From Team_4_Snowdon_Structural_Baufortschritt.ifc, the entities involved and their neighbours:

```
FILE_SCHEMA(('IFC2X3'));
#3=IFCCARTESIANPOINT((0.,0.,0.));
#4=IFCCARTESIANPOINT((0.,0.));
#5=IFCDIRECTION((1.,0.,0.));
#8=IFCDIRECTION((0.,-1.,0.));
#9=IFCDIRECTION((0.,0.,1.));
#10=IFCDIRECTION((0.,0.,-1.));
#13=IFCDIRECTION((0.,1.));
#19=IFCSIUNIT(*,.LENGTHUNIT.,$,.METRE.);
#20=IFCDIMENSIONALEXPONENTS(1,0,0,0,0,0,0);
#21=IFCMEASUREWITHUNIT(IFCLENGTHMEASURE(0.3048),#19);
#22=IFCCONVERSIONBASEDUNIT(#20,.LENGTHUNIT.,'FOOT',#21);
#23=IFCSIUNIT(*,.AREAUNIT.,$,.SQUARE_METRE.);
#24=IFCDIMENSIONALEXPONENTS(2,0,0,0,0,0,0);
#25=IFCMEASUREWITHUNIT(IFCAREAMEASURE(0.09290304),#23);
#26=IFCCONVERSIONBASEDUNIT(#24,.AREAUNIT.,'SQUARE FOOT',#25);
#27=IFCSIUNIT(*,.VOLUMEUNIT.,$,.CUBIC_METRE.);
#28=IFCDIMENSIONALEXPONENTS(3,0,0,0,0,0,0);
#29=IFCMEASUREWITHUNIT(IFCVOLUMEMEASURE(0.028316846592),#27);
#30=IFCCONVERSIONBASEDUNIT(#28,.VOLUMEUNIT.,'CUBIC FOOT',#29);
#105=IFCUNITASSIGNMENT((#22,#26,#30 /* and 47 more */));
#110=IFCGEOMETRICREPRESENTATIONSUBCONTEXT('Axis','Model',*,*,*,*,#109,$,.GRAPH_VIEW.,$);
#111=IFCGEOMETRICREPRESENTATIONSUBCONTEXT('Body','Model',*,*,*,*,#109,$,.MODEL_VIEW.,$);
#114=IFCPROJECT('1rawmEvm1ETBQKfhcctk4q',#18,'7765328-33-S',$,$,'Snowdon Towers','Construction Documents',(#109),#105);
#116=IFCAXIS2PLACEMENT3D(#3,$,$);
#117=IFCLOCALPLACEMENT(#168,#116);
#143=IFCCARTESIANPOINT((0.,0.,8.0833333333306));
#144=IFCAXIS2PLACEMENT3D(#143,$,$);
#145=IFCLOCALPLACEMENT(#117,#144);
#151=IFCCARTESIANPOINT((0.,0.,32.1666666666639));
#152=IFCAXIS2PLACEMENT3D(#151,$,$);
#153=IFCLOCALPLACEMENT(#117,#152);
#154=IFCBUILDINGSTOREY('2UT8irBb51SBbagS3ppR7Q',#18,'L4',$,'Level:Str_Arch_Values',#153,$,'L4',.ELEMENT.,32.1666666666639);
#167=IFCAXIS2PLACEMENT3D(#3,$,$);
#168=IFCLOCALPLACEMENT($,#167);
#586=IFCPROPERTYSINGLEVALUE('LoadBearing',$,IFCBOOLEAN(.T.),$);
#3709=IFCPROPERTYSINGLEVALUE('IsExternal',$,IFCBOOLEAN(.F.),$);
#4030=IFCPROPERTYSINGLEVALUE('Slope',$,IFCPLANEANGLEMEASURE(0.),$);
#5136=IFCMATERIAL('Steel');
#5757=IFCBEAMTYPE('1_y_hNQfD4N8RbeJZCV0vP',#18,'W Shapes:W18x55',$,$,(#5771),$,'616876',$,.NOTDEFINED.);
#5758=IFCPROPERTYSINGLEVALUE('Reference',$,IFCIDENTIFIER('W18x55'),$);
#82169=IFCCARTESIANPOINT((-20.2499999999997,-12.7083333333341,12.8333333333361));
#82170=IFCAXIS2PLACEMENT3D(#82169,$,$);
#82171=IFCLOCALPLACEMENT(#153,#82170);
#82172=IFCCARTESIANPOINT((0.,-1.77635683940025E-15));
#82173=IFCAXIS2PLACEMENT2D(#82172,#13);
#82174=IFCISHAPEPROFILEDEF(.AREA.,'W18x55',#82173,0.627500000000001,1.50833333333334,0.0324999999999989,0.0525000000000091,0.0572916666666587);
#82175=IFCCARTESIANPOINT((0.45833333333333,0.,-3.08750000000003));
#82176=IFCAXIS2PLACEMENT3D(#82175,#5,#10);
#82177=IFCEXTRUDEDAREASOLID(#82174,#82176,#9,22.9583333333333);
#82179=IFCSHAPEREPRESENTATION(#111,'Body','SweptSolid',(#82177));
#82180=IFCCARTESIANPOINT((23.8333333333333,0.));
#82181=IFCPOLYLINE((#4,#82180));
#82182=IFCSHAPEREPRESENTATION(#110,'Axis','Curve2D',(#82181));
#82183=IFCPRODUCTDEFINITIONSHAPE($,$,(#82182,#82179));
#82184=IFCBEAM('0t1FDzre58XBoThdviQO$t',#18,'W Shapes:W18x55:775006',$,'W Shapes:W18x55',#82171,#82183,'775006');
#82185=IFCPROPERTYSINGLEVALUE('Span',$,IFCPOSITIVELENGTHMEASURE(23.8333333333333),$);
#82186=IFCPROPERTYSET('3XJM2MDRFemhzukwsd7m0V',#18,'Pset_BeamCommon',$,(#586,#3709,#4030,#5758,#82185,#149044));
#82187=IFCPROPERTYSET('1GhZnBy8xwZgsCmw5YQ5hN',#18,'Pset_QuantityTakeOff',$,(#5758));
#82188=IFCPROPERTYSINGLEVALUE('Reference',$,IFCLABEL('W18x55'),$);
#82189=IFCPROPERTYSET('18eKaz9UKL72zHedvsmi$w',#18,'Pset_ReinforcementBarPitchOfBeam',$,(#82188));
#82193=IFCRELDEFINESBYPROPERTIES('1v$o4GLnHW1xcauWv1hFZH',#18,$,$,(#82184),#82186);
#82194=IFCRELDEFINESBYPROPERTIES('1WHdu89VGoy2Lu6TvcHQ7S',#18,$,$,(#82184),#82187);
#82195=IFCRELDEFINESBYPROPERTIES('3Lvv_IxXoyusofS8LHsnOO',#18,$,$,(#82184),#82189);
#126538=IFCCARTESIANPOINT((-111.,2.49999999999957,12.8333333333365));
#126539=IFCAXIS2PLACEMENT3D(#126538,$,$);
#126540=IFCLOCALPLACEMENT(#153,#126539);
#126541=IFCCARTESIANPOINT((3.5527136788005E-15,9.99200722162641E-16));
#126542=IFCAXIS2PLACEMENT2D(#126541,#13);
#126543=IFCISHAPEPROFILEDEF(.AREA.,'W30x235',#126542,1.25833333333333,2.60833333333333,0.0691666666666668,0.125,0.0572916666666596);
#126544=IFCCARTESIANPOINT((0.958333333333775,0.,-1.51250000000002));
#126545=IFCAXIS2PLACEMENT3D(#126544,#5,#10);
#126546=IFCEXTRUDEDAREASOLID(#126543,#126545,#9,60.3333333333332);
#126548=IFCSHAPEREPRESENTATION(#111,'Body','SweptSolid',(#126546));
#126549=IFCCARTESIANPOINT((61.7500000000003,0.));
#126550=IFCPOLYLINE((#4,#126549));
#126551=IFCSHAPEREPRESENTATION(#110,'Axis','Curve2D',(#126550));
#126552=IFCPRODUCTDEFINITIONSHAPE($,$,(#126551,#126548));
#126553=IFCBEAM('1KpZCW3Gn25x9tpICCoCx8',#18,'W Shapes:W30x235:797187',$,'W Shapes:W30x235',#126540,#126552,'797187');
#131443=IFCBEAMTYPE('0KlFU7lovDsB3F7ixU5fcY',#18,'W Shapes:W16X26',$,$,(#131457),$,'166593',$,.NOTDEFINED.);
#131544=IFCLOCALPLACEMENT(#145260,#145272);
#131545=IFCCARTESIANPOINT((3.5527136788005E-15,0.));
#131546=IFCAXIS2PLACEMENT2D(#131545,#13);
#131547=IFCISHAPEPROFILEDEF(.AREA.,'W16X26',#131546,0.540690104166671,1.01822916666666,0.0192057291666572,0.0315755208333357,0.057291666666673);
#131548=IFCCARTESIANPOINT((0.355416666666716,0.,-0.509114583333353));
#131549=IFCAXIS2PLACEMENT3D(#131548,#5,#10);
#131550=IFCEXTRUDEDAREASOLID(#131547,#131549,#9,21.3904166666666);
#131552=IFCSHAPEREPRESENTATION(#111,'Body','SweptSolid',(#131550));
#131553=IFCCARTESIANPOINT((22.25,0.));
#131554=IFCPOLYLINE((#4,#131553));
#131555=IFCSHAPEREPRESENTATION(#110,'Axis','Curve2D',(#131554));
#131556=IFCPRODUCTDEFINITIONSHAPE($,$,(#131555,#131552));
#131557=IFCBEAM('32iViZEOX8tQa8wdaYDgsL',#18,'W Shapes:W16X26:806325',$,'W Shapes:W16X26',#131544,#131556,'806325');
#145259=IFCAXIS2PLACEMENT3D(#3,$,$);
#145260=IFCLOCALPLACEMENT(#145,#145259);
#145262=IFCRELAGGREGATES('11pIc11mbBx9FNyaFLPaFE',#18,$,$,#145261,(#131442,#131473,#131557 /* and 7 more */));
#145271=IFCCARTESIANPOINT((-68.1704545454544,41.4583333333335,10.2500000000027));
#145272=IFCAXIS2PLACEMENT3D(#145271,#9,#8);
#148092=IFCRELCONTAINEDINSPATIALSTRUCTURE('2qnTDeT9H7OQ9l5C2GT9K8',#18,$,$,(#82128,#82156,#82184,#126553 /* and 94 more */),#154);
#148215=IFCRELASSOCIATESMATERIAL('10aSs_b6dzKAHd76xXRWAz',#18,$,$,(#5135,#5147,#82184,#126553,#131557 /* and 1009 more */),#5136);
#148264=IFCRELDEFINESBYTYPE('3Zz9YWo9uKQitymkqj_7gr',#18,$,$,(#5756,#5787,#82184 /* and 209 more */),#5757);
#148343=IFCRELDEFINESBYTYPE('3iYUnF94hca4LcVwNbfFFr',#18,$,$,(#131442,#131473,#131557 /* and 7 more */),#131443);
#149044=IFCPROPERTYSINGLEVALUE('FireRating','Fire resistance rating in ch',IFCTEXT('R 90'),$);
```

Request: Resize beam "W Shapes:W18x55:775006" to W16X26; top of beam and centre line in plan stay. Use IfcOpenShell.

```python
import ifcopenshell
import ifcopenshell.api.pset
import ifcopenshell.api.type
import ifcopenshell.util.element
import ifcopenshell.util.representation

model = ifcopenshell.open("Team_4_Snowdon_Structural_Baufortschritt.ifc")

member = model.by_guid("0t1FDzre58XBoThdviQO$t")
source = next(p for p in model.by_type("IfcIShapeProfileDef") if p.ProfileName == "W16X26")

body = ifcopenshell.util.representation.get_representation(member, "Model", "Body")
solid = body.Items[0]
old_profile = solid.SweptArea

# Copy the section's sizes but keep this member's own profile position.
profile = ifcopenshell.util.element.copy(model, source)
# Profiles are centred, so shift by half the change in depth to hold the top.
shift = (old_profile.OverallDepth - profile.OverallDepth) / 2
x, y = old_profile.Position.Location.Coordinates
up = (-1.0, 0.0)  # upwards, in the solid's own plane
location = model.createIfcCartesianPoint((x + up[0] * shift, y + up[1] * shift))
profile.Position = model.createIfcAxis2Placement2D(location, old_profile.Position.RefDirection)
solid.SweptArea = profile
if not model.get_total_inverses(old_profile):
    ifcopenshell.util.element.remove_deep2(model, old_profile)

new_type = model.by_id(131443)
ifcopenshell.api.type.assign_type(
    model, related_objects=[member], relating_type=new_type, should_map_representations=False
)
member.Name = member.Name.replace("W18x55", "W16X26")
member.ObjectType = "W Shapes:W16X26"
pset = model.by_id(ifcopenshell.util.element.get_pset(member, "Pset_BeamCommon", should_inherit=False)["id"])
ifcopenshell.api.pset.edit_pset(model, pset=pset, properties={"Reference": "W16X26"})
pset = model.by_id(ifcopenshell.util.element.get_pset(member, "Pset_QuantityTakeOff", should_inherit=False)["id"])
ifcopenshell.api.pset.edit_pset(model, pset=pset, properties={"Reference": "W16X26"})
pset = model.by_id(ifcopenshell.util.element.get_pset(member, "Pset_ReinforcementBarPitchOfBeam", should_inherit=False)["id"])
ifcopenshell.api.pset.edit_pset(model, pset=pset, properties={"Reference": "W16X26"})

print(solid.SweptArea)

model.write("Team_4_Snowdon_Structural_Baufortschritt_edited.ifc")
```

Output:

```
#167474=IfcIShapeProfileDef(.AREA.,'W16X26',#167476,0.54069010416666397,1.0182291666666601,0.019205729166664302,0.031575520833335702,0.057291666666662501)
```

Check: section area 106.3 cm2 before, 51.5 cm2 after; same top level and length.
